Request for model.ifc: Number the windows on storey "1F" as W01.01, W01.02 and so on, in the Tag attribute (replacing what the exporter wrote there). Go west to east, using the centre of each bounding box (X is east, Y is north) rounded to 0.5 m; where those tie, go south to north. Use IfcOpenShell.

First a look at what the model holds.

```python
import ifcopenshell
import ifcopenshell.util.element
import ifcopenshell.util.placement

model = ifcopenshell.open("model.ifc")
print(model.schema)
storey = next(s for s in model.by_type("IfcBuildingStorey") if s.Name == "1F")
windows = [e for e in ifcopenshell.util.element.get_decomposition(storey) if e.is_a("IfcWindow")]
for e in sorted(windows, key=lambda e: e.id()):
    origin = ifcopenshell.util.placement.get_local_placement(e.ObjectPlacement)[:3, 3]
    print(e.id(), e.Tag, e.Name, origin.round(2) + 0.0, sep=" | ")
```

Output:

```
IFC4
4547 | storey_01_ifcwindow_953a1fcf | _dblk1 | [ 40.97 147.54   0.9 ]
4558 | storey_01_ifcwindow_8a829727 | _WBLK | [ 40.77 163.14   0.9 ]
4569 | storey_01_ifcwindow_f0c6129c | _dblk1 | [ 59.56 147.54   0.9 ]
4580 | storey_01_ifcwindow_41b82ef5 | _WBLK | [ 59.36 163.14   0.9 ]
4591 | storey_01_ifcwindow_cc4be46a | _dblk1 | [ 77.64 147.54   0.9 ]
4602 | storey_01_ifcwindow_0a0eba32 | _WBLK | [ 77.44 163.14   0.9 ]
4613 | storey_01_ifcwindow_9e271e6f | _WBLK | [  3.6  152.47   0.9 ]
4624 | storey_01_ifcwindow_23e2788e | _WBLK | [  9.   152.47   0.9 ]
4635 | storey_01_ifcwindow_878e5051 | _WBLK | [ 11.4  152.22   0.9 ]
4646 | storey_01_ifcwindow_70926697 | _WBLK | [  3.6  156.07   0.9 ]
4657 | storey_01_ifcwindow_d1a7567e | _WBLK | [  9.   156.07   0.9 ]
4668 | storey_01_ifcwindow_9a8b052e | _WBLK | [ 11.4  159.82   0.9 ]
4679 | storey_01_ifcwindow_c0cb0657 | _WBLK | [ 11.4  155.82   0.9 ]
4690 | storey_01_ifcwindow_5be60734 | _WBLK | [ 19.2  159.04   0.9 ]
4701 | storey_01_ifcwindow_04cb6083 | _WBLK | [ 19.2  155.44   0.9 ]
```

```python
import ifcopenshell
import ifcopenshell.geom
import ifcopenshell.util.element
import ifcopenshell.util.shape

model = ifcopenshell.open("model.ifc")
settings = ifcopenshell.geom.settings()
settings.set("use-world-coords", True)


def centre(element):
    shape = ifcopenshell.geom.create_shape(settings, element)
    return ifcopenshell.util.shape.get_bbox_centroid(shape.geometry)


storey = next(s for s in model.by_type("IfcBuildingStorey") if s.Name == "1F")
windows = [e for e in ifcopenshell.util.element.get_decomposition(storey) if e.is_a("IfcWindow")]

# Insertion points can sit at a corner or the storey origin, so sort by the geometry (in metres).
centres = {e: centre(e) for e in windows}
windows.sort(key=lambda e: (round(centres[e][0] / 0.5), centres[e][1]))

for i, e in enumerate(windows, start=1):
    number = f"W01.{i:02d}"
    e.Tag = number
    print(e.id(), number)

model.write("model_rev.ifc")
```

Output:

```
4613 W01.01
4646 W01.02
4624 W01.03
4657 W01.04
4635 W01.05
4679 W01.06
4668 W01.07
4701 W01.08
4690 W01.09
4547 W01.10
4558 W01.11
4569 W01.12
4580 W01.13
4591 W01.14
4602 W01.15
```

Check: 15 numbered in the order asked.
